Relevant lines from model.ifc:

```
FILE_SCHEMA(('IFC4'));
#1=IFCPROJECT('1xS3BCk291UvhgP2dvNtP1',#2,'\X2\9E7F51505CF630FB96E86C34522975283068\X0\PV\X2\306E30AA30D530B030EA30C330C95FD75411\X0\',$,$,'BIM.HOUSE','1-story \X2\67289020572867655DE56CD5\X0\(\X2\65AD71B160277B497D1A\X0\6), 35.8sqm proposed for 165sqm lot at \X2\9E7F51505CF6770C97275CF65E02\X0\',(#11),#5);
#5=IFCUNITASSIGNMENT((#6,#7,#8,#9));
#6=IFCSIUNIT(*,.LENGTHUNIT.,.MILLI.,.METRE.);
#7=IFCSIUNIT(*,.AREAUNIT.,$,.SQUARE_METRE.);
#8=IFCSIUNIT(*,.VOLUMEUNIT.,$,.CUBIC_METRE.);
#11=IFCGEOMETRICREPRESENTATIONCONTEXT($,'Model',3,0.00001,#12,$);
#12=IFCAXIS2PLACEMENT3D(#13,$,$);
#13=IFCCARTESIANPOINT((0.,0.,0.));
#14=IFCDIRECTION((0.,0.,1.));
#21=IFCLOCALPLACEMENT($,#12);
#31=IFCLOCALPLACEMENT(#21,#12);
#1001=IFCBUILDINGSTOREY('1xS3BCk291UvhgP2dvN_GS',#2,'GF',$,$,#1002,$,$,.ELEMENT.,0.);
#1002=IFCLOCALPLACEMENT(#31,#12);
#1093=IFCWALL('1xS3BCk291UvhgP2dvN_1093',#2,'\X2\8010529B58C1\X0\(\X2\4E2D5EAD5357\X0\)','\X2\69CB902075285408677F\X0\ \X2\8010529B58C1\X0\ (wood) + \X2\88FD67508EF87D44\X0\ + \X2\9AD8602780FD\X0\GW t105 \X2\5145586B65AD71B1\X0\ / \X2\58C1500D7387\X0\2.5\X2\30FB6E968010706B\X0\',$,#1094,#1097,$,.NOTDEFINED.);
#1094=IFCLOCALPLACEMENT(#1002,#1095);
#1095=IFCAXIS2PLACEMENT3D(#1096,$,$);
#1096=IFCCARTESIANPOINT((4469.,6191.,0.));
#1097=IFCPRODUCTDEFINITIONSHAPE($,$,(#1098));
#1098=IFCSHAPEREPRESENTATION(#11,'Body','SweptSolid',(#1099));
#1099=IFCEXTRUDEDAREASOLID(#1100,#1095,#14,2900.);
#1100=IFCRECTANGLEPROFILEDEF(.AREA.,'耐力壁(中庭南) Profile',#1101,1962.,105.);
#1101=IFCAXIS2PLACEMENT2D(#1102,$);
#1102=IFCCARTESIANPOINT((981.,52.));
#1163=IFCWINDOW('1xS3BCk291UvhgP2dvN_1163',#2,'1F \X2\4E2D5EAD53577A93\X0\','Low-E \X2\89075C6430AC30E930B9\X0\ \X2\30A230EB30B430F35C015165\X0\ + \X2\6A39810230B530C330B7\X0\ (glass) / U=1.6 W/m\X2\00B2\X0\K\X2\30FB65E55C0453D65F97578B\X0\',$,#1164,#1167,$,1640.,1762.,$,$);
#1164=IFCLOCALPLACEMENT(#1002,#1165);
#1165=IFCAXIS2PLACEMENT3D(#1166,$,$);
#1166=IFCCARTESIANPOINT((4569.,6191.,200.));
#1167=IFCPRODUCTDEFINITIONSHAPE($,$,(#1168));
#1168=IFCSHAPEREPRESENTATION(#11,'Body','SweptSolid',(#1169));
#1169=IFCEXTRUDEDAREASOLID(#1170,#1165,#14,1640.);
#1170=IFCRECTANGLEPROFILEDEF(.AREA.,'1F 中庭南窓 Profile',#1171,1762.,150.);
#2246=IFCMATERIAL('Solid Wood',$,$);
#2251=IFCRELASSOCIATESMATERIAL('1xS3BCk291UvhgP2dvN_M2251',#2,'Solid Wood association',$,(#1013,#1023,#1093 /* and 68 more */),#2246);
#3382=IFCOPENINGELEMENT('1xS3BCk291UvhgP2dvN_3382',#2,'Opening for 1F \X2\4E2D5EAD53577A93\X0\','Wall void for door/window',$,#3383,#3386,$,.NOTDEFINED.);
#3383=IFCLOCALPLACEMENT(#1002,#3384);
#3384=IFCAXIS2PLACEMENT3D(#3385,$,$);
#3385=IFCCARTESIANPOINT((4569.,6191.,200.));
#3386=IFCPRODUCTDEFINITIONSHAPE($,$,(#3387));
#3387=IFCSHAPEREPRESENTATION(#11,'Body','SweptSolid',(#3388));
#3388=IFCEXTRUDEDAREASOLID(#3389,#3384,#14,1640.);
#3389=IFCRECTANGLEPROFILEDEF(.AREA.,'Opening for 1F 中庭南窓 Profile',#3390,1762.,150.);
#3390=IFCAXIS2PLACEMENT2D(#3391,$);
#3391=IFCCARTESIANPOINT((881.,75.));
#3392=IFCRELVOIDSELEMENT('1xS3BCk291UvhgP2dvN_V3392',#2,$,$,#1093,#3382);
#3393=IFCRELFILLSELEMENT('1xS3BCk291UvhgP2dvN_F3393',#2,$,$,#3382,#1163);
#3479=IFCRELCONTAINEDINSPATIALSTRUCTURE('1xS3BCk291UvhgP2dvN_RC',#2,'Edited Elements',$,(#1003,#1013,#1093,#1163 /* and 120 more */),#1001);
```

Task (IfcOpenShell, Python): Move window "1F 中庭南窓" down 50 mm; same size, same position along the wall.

```python
import numpy as np
import ifcopenshell
import ifcopenshell.api.geometry
import ifcopenshell.util.placement
import ifcopenshell.util.unit

model = ifcopenshell.open("model.ifc")
unit_scale = ifcopenshell.util.unit.calculate_unit_scale(model)

window = model.by_guid("1xS3BCk291UvhgP2dvN_1163")
opening = window.FillsVoids[0].RelatingOpeningElement
dz = -50.0

shift = np.array([0.0, 0.0, dz])
# The window is not placed relative to its opening, so move both.
for product in (opening, window):
    matrix = ifcopenshell.util.placement.get_local_placement(product.ObjectPlacement)
    matrix[:3, 3] += shift
    ifcopenshell.api.geometry.edit_object_placement(model, product=product, matrix=matrix, is_si=False)

print(f"moved by {dz * unit_scale:+.3f} m")

model.write("model_updated.ifc")
```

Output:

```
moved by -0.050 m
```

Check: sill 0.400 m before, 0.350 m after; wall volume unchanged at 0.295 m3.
